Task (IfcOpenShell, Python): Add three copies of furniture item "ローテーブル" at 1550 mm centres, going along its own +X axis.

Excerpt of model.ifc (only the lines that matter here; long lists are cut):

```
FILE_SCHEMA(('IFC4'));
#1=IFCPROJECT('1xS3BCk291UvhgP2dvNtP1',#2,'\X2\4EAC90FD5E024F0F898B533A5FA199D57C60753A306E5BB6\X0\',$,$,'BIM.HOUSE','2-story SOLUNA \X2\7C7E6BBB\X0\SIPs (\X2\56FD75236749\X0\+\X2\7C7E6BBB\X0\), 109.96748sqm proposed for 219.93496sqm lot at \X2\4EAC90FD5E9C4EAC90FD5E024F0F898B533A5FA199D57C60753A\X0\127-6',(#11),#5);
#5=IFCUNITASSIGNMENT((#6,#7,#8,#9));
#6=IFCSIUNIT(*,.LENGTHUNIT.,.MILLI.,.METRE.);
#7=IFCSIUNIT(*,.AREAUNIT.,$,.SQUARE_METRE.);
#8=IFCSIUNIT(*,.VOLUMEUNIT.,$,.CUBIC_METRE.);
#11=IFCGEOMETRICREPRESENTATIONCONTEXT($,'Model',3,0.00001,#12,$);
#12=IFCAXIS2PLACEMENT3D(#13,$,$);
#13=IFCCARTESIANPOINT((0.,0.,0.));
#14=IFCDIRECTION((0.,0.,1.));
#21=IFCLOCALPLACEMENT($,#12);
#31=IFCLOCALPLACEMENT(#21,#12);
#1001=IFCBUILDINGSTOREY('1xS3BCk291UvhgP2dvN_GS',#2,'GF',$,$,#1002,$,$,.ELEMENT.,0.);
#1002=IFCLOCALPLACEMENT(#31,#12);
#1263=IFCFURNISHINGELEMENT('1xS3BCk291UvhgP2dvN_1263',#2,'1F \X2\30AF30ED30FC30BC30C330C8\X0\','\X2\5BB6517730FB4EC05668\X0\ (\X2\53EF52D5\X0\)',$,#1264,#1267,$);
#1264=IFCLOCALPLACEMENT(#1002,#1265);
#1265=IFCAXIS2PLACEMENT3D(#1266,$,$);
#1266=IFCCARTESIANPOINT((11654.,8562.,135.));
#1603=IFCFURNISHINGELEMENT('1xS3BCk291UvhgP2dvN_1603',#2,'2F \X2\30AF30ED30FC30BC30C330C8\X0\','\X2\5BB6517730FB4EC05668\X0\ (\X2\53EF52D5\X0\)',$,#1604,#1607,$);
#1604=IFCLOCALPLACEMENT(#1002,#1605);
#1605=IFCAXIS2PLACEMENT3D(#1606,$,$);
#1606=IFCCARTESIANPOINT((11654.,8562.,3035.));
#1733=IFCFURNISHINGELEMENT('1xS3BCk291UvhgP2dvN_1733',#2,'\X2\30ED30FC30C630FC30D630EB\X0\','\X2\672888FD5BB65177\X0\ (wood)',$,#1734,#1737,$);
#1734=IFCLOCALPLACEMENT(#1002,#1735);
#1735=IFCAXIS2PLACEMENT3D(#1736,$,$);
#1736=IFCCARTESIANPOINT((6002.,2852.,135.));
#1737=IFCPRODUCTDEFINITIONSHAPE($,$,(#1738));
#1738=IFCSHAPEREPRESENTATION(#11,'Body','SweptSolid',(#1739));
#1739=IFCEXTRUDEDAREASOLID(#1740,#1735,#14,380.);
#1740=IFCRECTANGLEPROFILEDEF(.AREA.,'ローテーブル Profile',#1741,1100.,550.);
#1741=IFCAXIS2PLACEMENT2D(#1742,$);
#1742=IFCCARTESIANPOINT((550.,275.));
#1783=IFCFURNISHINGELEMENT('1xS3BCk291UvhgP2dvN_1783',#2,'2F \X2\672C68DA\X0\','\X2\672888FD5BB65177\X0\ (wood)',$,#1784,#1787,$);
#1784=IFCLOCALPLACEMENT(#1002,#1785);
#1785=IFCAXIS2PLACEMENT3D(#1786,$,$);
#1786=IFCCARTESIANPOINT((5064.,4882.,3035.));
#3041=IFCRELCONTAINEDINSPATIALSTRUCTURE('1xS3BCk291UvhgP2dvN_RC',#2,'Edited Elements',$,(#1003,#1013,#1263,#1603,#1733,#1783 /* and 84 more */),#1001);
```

```python
import ifcopenshell
import ifcopenshell.api.geometry
import ifcopenshell.api.root
import ifcopenshell.util.element
import ifcopenshell.util.placement
import ifcopenshell.util.unit

model = ifcopenshell.open("model.ifc")
unit_scale = ifcopenshell.util.unit.calculate_unit_scale(model)


def reuse_history(source, copy):
    """copy_class also copies each property set's owner history, people and application; keep the originals."""
    for rel in copy.IsDefinedBy:
        if rel.is_a("IfcRelDefinesByProperties") and (history := rel.RelatingPropertyDefinition.OwnerHistory):
            rel.RelatingPropertyDefinition.OwnerHistory = source.OwnerHistory
            ifcopenshell.util.element.remove_deep2(model, history)


source = model.by_guid("1xS3BCk291UvhgP2dvN_1733")
base = ifcopenshell.util.placement.get_local_placement(source.ObjectPlacement)
step = base[:3, 0] * 1.55 / unit_scale

for i in range(1, 4):
    copy = ifcopenshell.api.root.copy_class(model, product=source)
    copy.Representation = ifcopenshell.util.element.copy_deep(
        model, source.Representation, exclude=["IfcGeometricRepresentationContext", "IfcRepresentationMap"]
    )
    reuse_history(source, copy)
    matrix = base.copy()
    matrix[:3, 3] += i * step
    print("added at", matrix[:3, 3].round(3) + 0.0)
    ifcopenshell.api.geometry.edit_object_placement(model, product=copy, matrix=matrix, is_si=False)

model.write("model_edited.ifc")
```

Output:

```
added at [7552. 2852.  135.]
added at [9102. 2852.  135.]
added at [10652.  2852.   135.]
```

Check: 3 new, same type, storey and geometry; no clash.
